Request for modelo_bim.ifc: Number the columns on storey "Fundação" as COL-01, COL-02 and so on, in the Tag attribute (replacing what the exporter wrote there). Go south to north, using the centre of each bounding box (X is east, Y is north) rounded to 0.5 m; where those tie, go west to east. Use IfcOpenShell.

First a look at what the model holds.

```python
import ifcopenshell
import ifcopenshell.util.element
import ifcopenshell.util.placement

model = ifcopenshell.open("modelo_bim.ifc")
print(model.schema)
storey = next(s for s in model.by_type("IfcBuildingStorey") if s.Name == "Fundação")
columns = [e for e in ifcopenshell.util.element.get_decomposition(storey) if e.is_a("IfcColumn")]
for e in sorted(columns, key=lambda e: e.id()):
    origin = ifcopenshell.util.placement.get_local_placement(e.ObjectPlacement)[:3, 3]
    print(e.id(), e.Tag, e.Name, origin.round(2) + 0.0, sep=" | ")
```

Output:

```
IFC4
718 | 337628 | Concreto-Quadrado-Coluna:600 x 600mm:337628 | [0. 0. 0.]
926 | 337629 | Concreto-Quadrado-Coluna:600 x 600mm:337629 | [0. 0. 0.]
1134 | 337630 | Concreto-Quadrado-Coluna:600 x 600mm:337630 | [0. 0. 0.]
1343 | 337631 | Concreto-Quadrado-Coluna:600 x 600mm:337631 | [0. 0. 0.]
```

```python
import ifcopenshell
import ifcopenshell.geom
import ifcopenshell.util.element
import ifcopenshell.util.shape

model = ifcopenshell.open("modelo_bim.ifc")
settings = ifcopenshell.geom.settings()
settings.set("use-world-coords", True)


def centre(element):
    shape = ifcopenshell.geom.create_shape(settings, element)
    return ifcopenshell.util.shape.get_bbox_centroid(shape.geometry)


storey = next(s for s in model.by_type("IfcBuildingStorey") if s.Name == "Fundação")
columns = [e for e in ifcopenshell.util.element.get_decomposition(storey) if e.is_a("IfcColumn")]

# Insertion points can sit at a corner or the storey origin, so sort by the geometry (in metres).
centres = {e: centre(e) for e in columns}
columns.sort(key=lambda e: (round(centres[e][1] / 0.5), centres[e][0]))

for i, e in enumerate(columns, start=1):
    number = f"COL-{i:02d}"
    e.Tag = number
    print(e.id(), number)

model.write("modelo_bim_v2.ifc")
```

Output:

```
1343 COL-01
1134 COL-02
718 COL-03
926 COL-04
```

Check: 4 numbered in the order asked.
